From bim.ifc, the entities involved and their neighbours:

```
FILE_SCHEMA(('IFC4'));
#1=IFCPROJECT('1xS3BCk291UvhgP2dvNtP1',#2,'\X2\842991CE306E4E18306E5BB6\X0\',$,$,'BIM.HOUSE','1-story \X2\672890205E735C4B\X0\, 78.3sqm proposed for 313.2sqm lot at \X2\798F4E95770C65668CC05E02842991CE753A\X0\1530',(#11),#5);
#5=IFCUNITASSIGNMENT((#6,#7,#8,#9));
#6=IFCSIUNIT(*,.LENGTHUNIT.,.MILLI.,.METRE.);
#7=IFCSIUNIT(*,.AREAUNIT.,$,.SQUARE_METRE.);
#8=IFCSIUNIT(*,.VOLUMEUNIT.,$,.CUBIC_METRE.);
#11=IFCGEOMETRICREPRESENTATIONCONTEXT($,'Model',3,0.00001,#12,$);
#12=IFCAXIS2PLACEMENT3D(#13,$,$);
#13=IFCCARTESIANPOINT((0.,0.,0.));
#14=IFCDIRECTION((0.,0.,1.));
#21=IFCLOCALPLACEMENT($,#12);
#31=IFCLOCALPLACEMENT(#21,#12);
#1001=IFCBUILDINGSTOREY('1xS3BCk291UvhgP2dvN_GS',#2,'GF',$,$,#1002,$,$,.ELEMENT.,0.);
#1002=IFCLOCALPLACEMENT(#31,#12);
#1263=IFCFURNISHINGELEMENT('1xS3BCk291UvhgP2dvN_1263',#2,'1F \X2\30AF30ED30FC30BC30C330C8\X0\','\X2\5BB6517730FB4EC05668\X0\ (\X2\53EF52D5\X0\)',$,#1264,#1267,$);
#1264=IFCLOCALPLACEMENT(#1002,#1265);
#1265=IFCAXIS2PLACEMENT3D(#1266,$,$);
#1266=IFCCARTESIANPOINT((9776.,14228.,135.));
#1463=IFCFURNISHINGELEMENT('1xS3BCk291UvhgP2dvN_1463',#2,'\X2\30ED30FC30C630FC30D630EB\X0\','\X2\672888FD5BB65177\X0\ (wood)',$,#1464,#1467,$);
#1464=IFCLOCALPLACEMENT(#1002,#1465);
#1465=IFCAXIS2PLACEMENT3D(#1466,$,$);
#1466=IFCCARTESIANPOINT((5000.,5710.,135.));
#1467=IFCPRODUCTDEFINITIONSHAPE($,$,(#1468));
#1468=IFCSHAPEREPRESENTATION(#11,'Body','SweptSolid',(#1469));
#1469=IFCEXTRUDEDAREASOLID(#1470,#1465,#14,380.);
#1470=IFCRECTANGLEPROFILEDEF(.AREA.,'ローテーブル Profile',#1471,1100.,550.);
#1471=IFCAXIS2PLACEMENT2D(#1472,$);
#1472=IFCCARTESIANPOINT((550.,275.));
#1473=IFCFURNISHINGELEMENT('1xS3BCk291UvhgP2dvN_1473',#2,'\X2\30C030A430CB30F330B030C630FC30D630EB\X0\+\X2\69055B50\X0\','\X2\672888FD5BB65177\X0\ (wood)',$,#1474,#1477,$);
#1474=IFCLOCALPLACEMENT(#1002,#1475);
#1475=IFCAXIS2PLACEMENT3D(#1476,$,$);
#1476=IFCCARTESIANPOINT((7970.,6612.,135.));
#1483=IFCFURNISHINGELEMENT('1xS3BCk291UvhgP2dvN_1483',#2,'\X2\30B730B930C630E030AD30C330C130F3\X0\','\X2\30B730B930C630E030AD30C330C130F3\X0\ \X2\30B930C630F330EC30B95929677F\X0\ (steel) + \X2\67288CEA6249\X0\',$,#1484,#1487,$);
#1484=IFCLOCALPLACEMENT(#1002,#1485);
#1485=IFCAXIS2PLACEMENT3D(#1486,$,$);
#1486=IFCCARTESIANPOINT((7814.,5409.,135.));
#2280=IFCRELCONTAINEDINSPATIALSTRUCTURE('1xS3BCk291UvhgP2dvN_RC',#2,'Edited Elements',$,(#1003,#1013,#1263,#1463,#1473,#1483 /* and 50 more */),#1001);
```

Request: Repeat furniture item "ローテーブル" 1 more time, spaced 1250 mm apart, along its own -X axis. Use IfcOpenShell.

```python
import ifcopenshell
import ifcopenshell.api.geometry
import ifcopenshell.api.root
import ifcopenshell.util.element
import ifcopenshell.util.placement

model = ifcopenshell.open("bim.ifc")


def reuse_history(source, copy):
    """copy_class also copies each property set's owner history, people and application; keep the originals."""
    for rel in copy.IsDefinedBy:
        if rel.is_a("IfcRelDefinesByProperties") and (history := rel.RelatingPropertyDefinition.OwnerHistory):
            rel.RelatingPropertyDefinition.OwnerHistory = source.OwnerHistory
            ifcopenshell.util.element.remove_deep2(model, history)


source = model.by_guid("1xS3BCk291UvhgP2dvN_1463")
base = ifcopenshell.util.placement.get_local_placement(source.ObjectPlacement)
step = -base[:3, 0] * 1250.0

for i in range(1, 2):
    copy = ifcopenshell.api.root.copy_class(model, product=source)
    copy.Representation = ifcopenshell.util.element.copy_deep(
        model, source.Representation, exclude=["IfcGeometricRepresentationContext", "IfcRepresentationMap"]
    )
    reuse_history(source, copy)
    matrix = base.copy()
    matrix[:3, 3] += i * step
    print("added at", matrix[:3, 3].round(3) + 0.0)
    ifcopenshell.api.geometry.edit_object_placement(model, product=copy, matrix=matrix, is_si=False)

model.write("bim_rev.ifc")
```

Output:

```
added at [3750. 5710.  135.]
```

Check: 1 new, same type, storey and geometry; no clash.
